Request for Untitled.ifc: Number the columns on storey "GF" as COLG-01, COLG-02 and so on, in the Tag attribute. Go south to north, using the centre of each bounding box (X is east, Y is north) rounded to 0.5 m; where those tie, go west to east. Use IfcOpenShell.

First a look at what the model holds.

```python
import ifcopenshell
import ifcopenshell.util.element
import ifcopenshell.util.placement

model = ifcopenshell.open("Untitled.ifc")
print(model.schema)
storey = next(s for s in model.by_type("IfcBuildingStorey") if s.Name == "GF")
columns = [e for e in ifcopenshell.util.element.get_decomposition(storey) if e.is_a("IfcColumn")]
for e in sorted(columns, key=lambda e: e.id()):
    origin = ifcopenshell.util.placement.get_local_placement(e.ObjectPlacement)[:3, 3]
    print(e.id(), e.Tag, e.Name, origin.round(2) + 0.0, sep=" | ")
```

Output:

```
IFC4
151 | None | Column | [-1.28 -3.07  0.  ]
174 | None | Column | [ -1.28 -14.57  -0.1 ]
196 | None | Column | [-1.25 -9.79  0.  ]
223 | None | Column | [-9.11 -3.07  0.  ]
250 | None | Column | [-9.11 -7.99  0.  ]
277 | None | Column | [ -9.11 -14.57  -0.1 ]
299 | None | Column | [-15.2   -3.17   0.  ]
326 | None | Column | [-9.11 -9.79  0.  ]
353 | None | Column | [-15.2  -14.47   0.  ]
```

```python
import ifcopenshell
import ifcopenshell.geom
import ifcopenshell.util.element
import ifcopenshell.util.shape

model = ifcopenshell.open("Untitled.ifc")
settings = ifcopenshell.geom.settings()
settings.set("use-world-coords", True)


def centre(element):
    shape = ifcopenshell.geom.create_shape(settings, element)
    return ifcopenshell.util.shape.get_bbox_centroid(shape.geometry)


storey = next(s for s in model.by_type("IfcBuildingStorey") if s.Name == "GF")
columns = [e for e in ifcopenshell.util.element.get_decomposition(storey) if e.is_a("IfcColumn")]

# Insertion points can sit at a corner or the storey origin, so sort by the geometry (in metres).
centres = {e: centre(e) for e in columns}
columns.sort(key=lambda e: (round(centres[e][1] / 0.5), centres[e][0]))

for i, e in enumerate(columns, start=1):
    number = f"COLG-{i:02d}"
    e.Tag = number
    print(e.id(), number)

model.write("Untitled_updated.ifc")
```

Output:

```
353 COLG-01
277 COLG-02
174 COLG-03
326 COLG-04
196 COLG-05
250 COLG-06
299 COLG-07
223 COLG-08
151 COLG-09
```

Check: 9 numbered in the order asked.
